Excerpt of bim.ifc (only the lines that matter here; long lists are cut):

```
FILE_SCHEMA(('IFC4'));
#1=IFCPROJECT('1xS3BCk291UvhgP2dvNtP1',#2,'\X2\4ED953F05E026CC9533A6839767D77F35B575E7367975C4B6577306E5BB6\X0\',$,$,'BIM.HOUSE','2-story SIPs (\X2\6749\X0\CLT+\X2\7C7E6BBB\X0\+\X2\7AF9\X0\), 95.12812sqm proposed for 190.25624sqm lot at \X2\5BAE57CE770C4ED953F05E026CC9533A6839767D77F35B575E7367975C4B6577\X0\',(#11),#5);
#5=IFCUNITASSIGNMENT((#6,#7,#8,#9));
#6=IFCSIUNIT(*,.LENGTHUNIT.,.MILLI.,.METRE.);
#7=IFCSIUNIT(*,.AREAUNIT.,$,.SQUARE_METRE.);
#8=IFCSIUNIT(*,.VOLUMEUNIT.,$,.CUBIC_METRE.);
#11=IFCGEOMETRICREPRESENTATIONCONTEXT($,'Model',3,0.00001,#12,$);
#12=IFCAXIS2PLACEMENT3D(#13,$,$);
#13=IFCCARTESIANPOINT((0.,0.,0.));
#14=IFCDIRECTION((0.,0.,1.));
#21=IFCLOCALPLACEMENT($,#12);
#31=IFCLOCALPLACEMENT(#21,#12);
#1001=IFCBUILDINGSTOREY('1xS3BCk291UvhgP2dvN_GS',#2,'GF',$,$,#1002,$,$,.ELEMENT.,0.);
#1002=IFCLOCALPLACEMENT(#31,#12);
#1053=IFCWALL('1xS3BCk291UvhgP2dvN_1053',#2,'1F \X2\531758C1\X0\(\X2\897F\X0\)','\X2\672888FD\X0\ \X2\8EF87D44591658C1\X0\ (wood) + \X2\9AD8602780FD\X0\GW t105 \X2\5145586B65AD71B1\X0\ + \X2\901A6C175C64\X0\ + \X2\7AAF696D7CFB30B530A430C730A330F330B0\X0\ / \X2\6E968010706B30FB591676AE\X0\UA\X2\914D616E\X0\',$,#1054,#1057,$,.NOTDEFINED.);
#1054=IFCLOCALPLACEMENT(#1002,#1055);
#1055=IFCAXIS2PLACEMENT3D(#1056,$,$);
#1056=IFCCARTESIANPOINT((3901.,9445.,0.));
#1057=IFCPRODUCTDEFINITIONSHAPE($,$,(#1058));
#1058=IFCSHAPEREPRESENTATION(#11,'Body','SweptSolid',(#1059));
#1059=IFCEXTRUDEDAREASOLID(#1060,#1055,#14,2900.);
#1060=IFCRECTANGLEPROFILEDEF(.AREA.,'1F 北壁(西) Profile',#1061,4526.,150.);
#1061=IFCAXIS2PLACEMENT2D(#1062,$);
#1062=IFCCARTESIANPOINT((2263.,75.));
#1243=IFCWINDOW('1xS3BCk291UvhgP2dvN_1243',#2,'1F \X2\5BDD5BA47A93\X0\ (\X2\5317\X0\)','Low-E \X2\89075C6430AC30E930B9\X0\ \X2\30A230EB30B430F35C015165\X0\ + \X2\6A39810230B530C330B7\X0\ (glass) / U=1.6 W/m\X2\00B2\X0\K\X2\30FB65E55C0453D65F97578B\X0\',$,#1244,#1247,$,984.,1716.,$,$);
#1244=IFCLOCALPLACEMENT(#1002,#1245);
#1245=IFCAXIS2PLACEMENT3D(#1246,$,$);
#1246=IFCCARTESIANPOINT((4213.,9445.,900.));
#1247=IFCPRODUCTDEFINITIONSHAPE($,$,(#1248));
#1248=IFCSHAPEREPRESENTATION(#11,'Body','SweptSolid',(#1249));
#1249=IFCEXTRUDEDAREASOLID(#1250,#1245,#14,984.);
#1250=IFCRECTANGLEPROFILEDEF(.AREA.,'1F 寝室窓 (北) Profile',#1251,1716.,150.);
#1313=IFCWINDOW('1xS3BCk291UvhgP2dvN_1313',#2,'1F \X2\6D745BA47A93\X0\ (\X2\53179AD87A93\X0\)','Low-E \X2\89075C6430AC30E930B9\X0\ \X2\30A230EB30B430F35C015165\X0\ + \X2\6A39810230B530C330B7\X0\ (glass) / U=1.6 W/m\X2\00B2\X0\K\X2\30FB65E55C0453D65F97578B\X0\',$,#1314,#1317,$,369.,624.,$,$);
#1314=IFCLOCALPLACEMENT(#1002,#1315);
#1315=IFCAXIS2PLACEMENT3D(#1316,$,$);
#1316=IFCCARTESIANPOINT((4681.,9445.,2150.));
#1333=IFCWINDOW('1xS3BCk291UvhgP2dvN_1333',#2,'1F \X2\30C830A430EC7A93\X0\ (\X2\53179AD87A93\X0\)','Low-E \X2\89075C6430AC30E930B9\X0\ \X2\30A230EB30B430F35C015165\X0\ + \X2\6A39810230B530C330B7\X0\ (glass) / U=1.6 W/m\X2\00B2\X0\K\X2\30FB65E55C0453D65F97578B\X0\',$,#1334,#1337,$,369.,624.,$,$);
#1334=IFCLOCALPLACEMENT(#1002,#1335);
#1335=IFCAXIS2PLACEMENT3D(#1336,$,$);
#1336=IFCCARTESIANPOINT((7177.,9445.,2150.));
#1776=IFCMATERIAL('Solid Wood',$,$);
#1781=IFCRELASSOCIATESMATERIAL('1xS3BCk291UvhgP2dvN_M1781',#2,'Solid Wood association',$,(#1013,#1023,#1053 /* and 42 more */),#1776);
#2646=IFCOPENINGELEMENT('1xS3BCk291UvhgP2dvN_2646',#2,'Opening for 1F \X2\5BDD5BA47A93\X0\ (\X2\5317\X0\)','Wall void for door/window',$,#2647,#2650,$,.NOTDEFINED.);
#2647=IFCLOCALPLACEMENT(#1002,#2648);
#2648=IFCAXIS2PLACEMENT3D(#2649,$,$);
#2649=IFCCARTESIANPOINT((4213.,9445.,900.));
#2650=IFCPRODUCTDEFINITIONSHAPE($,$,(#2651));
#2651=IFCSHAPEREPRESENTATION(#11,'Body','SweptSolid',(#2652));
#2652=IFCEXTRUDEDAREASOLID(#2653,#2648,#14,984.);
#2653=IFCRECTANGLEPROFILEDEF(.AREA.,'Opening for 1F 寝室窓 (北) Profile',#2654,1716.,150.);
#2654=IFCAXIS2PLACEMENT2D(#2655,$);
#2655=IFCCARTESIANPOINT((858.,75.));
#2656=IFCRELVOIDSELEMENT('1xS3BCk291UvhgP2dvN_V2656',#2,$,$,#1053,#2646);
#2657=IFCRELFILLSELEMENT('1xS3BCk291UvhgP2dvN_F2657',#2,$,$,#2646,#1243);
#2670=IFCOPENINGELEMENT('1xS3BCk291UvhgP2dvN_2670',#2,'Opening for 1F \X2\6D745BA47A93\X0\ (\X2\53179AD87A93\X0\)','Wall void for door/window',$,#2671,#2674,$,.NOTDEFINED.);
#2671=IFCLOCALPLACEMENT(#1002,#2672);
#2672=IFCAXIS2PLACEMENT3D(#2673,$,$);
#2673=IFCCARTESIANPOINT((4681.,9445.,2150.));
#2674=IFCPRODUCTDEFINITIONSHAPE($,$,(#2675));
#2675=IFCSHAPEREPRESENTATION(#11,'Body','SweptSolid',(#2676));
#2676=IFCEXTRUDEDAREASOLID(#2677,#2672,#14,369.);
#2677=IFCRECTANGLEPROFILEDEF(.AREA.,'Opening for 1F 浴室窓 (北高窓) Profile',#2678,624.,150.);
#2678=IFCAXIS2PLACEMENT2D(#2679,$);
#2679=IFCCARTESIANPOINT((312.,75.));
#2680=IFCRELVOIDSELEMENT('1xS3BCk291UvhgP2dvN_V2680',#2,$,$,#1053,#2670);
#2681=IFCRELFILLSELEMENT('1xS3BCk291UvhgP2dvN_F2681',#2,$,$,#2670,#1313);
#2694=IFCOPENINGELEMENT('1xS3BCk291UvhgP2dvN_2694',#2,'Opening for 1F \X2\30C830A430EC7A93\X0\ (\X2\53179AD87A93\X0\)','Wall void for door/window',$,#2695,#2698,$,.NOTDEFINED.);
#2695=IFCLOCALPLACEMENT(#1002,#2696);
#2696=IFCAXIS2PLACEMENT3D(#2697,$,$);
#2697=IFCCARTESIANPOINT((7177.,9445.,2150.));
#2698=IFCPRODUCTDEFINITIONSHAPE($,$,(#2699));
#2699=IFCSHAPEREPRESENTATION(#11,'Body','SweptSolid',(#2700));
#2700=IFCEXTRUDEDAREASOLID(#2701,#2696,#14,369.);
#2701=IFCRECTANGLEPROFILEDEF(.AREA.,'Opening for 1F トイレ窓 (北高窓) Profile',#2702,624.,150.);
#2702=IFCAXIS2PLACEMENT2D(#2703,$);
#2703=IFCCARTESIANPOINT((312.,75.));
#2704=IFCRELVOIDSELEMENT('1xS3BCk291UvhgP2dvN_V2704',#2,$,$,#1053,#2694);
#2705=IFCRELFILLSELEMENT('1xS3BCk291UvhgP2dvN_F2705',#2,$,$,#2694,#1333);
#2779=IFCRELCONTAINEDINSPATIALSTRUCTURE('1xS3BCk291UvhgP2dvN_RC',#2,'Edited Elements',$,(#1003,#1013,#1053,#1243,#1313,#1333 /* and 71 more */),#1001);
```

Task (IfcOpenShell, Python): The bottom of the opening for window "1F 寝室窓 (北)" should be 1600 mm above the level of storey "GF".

```python
import numpy as np
import ifcopenshell
import ifcopenshell.api.geometry
import ifcopenshell.geom
import ifcopenshell.util.element
import ifcopenshell.util.placement
import ifcopenshell.util.shape
import ifcopenshell.util.unit

model = ifcopenshell.open("bim.ifc")
unit_scale = ifcopenshell.util.unit.calculate_unit_scale(model)

window = model.by_id(1243)
opening = window.FillsVoids[0].RelatingOpeningElement
storey = ifcopenshell.util.element.get_container(window, ifc_class="IfcBuildingStorey")
level = ifcopenshell.util.placement.get_local_placement(storey.ObjectPlacement)[2, 3]

# The opening's origin need not be at the sill, so measure its lowest point.
shape = ifcopenshell.geom.create_shape(ifcopenshell.geom.settings(), opening)
bottom = ifcopenshell.util.shape.get_shape_bottom_elevation(shape, shape.geometry) / unit_scale
dz = level + 1.6 / unit_scale - bottom

shift = np.array([0.0, 0.0, dz])
# The window is not placed relative to its opening, so move both.
for product in (opening, window):
    matrix = ifcopenshell.util.placement.get_local_placement(product.ObjectPlacement)
    matrix[:3, 3] += shift
    ifcopenshell.api.geometry.edit_object_placement(model, product=product, matrix=matrix, is_si=False)

print(f"moved by {dz * unit_scale:+.3f} m")

model.write("bim_v2.ifc")
```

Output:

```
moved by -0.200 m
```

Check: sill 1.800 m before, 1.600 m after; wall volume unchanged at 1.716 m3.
